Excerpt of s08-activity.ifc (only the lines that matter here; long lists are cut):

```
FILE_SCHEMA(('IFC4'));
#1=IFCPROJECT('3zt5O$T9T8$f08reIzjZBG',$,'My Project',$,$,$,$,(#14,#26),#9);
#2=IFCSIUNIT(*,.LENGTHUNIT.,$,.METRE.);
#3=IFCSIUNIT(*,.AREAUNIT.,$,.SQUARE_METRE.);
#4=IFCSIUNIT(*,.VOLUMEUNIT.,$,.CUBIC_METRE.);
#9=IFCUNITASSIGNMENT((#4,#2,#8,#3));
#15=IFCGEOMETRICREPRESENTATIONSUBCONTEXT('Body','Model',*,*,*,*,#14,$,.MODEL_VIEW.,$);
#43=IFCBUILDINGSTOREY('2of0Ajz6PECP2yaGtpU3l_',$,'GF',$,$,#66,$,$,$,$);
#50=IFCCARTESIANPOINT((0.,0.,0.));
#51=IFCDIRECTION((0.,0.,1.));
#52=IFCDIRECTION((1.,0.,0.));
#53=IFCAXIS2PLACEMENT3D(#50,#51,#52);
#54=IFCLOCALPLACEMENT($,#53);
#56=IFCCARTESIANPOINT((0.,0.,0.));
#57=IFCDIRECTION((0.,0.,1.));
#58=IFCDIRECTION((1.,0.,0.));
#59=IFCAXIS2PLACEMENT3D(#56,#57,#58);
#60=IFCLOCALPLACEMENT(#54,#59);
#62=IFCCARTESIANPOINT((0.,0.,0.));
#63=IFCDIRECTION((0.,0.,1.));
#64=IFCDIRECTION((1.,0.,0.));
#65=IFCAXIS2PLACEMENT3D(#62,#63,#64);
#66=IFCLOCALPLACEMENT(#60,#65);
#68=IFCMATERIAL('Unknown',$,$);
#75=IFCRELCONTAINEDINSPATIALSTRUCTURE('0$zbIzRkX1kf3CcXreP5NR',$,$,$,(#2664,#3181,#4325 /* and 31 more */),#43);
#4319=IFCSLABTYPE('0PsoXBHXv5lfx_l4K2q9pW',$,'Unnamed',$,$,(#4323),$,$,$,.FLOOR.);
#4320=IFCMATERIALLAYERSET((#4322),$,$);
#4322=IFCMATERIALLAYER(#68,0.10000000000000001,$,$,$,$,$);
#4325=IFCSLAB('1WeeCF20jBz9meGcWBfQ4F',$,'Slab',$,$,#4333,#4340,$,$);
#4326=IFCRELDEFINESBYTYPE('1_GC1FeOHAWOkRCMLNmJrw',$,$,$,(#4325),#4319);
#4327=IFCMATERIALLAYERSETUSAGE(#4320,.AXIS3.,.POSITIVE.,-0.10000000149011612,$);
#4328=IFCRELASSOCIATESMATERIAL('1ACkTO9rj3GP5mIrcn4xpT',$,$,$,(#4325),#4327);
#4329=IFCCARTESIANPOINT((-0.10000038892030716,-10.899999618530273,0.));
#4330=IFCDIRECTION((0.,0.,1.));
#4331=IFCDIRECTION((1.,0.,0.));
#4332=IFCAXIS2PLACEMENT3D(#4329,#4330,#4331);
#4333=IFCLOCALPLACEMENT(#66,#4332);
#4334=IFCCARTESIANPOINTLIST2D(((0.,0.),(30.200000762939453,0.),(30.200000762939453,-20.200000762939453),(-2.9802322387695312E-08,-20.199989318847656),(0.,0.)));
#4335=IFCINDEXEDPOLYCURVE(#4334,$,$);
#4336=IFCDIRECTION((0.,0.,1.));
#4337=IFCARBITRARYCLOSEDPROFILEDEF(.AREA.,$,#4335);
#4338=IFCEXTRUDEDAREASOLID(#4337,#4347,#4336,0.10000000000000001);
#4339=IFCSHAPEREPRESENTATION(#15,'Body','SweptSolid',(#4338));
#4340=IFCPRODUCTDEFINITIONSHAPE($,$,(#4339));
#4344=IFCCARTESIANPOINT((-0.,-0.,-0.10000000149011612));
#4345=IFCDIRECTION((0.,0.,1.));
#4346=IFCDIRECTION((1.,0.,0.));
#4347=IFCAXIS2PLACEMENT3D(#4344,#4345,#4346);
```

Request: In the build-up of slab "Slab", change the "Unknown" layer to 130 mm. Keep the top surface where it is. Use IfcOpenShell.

```python
import ifcopenshell
import ifcopenshell.util.element
import ifcopenshell.util.representation

model = ifcopenshell.open("s08-activity.ifc")

layer_set = model.by_id(4320)
layer = next(l for l in layer_set.MaterialLayers if l.Material and l.Material.Name == "Unknown")
change = 0.13 - layer.LayerThickness
layer.LayerThickness += change

# Geometry does not follow the layer set by itself.
slabs = [e for e in ifcopenshell.util.element.get_elements_by_material(model, layer_set) if e.is_a("IfcSlab")]
for slab in sorted(slabs, key=lambda e: e.id()):
    body = ifcopenshell.util.representation.get_representation(slab, "Model", "Body")
    solid = body.Items[0]
    old_depth = solid.Depth
    solid.Depth += change
    # Extruded upwards: lower the start of the extrusion so the top stays.
    x, y, z = solid.Position.Location.Coordinates
    solid.Position.Location = model.createIfcCartesianPoint((x, y, z - change))
    print(slab.id(), f"{old_depth:g} -> {solid.Depth:g}")

# The layers are counted up from the underside, which has moved.
for usage in {ifcopenshell.util.element.get_material(slab) for slab in slabs}:
    usage.OffsetFromReferenceLine -= change

model.write("s08-activity_edited.ifc")
```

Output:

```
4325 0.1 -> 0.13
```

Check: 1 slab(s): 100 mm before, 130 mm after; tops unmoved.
